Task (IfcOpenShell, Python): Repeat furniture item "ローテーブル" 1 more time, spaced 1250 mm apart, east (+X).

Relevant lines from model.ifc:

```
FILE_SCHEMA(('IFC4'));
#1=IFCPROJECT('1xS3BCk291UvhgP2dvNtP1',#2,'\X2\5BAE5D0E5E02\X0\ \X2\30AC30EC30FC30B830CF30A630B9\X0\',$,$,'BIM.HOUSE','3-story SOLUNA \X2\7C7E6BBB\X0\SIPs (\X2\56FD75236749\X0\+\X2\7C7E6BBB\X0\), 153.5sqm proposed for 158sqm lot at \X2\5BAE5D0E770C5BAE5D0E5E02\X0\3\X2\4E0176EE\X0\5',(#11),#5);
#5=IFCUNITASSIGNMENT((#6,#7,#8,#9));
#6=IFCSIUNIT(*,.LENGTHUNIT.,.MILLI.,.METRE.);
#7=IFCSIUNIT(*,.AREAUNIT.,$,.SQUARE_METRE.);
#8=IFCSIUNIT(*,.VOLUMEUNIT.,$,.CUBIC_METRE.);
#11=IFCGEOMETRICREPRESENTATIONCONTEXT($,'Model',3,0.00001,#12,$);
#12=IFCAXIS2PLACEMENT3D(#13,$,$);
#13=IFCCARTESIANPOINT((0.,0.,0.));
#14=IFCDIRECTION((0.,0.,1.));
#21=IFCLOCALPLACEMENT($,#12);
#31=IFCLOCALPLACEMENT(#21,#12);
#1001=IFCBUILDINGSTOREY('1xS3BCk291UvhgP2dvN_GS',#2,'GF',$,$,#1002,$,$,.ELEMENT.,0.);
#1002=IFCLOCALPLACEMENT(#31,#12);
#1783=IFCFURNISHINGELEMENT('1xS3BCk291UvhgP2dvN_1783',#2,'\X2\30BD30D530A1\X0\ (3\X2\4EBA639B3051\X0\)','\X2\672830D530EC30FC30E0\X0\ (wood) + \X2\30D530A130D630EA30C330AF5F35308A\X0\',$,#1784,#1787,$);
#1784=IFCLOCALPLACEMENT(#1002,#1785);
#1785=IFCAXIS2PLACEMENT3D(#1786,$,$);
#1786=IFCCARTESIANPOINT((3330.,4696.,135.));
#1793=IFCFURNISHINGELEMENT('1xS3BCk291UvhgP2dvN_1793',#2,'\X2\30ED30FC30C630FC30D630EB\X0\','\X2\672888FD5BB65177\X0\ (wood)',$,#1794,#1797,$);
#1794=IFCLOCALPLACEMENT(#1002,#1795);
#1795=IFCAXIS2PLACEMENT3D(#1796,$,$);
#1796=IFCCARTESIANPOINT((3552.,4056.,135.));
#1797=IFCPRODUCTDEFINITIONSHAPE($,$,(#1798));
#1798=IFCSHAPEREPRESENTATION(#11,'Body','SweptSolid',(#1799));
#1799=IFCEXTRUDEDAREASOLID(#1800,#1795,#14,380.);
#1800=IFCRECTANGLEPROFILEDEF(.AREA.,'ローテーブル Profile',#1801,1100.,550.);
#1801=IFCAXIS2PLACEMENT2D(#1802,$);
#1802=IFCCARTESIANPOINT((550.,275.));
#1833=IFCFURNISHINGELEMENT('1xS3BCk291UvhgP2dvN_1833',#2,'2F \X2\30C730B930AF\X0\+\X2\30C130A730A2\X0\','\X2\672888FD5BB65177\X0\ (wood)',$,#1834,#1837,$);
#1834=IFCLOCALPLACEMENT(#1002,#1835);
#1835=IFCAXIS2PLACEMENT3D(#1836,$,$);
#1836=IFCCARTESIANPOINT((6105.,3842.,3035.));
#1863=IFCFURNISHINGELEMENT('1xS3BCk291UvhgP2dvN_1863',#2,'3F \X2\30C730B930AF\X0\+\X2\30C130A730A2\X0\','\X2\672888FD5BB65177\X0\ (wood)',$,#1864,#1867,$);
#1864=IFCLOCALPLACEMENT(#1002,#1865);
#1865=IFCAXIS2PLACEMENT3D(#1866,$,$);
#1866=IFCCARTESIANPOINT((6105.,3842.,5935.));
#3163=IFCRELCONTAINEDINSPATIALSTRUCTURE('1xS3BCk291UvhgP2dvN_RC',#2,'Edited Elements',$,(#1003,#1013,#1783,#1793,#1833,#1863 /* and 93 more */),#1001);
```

```python
import numpy as np
import ifcopenshell
import ifcopenshell.api.geometry
import ifcopenshell.api.root
import ifcopenshell.util.element
import ifcopenshell.util.placement

model = ifcopenshell.open("model.ifc")


def reuse_history(source, copy):
    """copy_class also copies each property set's owner history, people and application; keep the originals."""
    for rel in copy.IsDefinedBy:
        if rel.is_a("IfcRelDefinesByProperties") and (history := rel.RelatingPropertyDefinition.OwnerHistory):
            rel.RelatingPropertyDefinition.OwnerHistory = source.OwnerHistory
            ifcopenshell.util.element.remove_deep2(model, history)


source = model.by_guid("1xS3BCk291UvhgP2dvN_1793")
base = ifcopenshell.util.placement.get_local_placement(source.ObjectPlacement)
step = np.array([1.0, 0.0, 0.0]) * 1250.0

for i in range(1, 2):
    copy = ifcopenshell.api.root.copy_class(model, product=source)
    copy.Representation = ifcopenshell.util.element.copy_deep(
        model, source.Representation, exclude=["IfcGeometricRepresentationContext", "IfcRepresentationMap"]
    )
    reuse_history(source, copy)
    matrix = base.copy()
    matrix[:3, 3] += i * step
    print("added at", matrix[:3, 3].round(3) + 0.0)
    ifcopenshell.api.geometry.edit_object_placement(model, product=copy, matrix=matrix, is_si=False)

model.write("model_rev.ifc")
```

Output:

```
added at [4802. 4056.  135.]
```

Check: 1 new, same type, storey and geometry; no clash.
